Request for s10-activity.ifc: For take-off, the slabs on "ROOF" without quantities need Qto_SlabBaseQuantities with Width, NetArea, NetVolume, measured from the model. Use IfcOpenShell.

First a look at what the model holds.

```python
import ifcopenshell
import ifcopenshell.util.element
import ifcopenshell.util.unit

model = ifcopenshell.open("s10-activity.ifc")
print(model.schema)
for unit_type in ("LENGTHUNIT", "AREAUNIT", "VOLUMEUNIT"):
    print(unit_type, ifcopenshell.util.unit.calculate_unit_scale(model, unit_type))
storey = next(s for s in model.by_type("IfcBuildingStorey") if s.Name == "ROOF")
slabs = [e for e in ifcopenshell.util.element.get_decomposition(storey) if e.is_a("IfcSlab")]
for e in sorted(slabs, key=lambda e: e.id()):
    print(e.id(), e.is_a(), e.Name, list(ifcopenshell.util.element.get_psets(e, qtos_only=True)), sep=" | ")
```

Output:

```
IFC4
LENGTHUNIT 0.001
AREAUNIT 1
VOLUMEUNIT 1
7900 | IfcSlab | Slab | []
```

```python
import ifcopenshell
import ifcopenshell.api.pset
import ifcopenshell.geom
import ifcopenshell.util.element
import ifcopenshell.util.shape
import ifcopenshell.util.unit

model = ifcopenshell.open("s10-activity.ifc")
unit_scale = ifcopenshell.util.unit.calculate_unit_scale(model)
area_scale = ifcopenshell.util.unit.calculate_unit_scale(model, "AREAUNIT")
volume_scale = ifcopenshell.util.unit.calculate_unit_scale(model, "VOLUMEUNIT")
settings = ifcopenshell.geom.settings()

storey = next(s for s in model.by_type("IfcBuildingStorey") if s.Name == "ROOF")
slabs = [e for e in ifcopenshell.util.element.get_decomposition(storey) if e.is_a("IfcSlab")]

for e in sorted(slabs, key=lambda e: e.id()):
    if ifcopenshell.util.element.get_psets(e, qtos_only=True, should_inherit=False):
        continue
    # Geometry comes back in metres, in the element's own axes.
    shape = ifcopenshell.geom.create_shape(settings, e)
    values = {
        "Width": ifcopenshell.util.shape.get_z(shape.geometry) / unit_scale,
        "NetArea": ifcopenshell.util.shape.get_footprint_area(shape.geometry) / area_scale,
        "NetVolume": ifcopenshell.util.shape.get_volume(shape.geometry) / volume_scale,
    }
    qto = ifcopenshell.api.pset.add_qto(model, product=e, name="Qto_SlabBaseQuantities")
    ifcopenshell.api.pset.edit_qto(model, qto=qto, properties=values)
    print(e.id(), {k: round(v, 3) for k, v in values.items()})

model.write("s10-activity-out.ifc")
```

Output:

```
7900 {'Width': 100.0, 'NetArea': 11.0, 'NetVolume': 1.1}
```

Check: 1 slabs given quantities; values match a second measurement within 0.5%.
